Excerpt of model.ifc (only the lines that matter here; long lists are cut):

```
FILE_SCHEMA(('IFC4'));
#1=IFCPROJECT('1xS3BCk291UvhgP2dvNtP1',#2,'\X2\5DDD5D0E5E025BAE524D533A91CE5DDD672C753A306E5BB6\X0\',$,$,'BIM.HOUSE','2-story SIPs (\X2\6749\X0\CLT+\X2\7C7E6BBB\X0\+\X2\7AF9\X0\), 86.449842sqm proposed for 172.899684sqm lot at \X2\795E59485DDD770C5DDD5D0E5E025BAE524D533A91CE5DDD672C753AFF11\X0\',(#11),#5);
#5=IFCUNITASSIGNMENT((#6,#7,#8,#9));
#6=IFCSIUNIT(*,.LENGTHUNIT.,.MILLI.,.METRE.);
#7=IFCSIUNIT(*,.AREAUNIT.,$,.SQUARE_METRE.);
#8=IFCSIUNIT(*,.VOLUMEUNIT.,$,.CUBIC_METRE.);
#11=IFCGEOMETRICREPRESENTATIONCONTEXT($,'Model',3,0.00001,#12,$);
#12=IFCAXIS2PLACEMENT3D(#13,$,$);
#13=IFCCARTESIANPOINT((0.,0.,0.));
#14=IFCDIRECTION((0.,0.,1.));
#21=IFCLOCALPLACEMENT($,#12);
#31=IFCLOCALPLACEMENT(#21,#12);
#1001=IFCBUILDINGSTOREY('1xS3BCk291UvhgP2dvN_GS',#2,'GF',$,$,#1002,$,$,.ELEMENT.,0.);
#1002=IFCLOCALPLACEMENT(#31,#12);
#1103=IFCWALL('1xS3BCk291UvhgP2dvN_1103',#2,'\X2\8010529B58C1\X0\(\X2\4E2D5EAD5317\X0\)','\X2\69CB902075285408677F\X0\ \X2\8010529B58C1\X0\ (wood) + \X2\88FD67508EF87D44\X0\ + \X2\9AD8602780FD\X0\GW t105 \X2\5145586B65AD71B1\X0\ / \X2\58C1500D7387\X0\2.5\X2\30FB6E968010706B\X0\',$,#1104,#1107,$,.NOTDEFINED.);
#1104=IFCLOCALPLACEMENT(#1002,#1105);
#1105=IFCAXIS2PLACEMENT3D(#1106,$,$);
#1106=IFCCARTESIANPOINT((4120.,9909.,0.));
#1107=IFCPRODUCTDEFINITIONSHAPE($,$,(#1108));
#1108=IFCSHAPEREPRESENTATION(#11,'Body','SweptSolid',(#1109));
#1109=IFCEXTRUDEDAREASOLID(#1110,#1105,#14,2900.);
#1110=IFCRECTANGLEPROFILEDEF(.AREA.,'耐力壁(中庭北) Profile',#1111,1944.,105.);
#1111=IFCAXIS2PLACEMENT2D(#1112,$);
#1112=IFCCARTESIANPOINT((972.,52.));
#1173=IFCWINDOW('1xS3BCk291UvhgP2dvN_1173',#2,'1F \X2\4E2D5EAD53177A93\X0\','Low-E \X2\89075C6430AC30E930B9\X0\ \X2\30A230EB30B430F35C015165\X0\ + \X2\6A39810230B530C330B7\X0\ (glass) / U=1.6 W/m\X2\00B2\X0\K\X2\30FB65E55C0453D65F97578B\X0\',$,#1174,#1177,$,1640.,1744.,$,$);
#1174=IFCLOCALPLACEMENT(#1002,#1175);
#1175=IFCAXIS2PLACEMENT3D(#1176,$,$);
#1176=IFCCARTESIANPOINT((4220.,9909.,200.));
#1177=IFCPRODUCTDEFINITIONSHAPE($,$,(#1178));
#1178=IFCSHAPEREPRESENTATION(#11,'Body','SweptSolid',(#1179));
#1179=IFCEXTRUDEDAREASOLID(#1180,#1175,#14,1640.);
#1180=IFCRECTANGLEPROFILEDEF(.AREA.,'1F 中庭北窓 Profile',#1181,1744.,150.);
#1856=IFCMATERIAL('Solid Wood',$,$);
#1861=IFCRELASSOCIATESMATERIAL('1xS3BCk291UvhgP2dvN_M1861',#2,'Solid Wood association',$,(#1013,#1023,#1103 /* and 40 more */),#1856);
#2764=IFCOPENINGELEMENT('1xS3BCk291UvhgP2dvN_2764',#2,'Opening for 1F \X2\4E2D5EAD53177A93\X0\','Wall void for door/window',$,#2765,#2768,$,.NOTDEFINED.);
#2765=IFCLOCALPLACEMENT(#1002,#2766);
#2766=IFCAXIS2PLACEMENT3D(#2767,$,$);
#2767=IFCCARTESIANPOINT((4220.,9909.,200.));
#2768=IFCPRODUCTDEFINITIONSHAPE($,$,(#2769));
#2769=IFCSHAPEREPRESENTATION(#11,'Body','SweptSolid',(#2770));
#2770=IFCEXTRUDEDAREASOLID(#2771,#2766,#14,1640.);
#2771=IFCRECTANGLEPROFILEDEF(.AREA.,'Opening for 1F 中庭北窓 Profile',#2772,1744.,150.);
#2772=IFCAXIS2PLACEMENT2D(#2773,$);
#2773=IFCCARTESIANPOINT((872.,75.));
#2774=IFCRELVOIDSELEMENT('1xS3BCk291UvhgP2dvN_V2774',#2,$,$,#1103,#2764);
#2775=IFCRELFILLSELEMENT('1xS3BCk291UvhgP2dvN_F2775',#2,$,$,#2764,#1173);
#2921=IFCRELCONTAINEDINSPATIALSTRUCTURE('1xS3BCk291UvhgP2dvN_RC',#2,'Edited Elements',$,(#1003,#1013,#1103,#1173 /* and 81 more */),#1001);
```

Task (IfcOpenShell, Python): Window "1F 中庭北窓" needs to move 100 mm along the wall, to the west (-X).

```python
import ifcopenshell
import ifcopenshell.api.geometry
import ifcopenshell.util.placement
import ifcopenshell.util.unit

model = ifcopenshell.open("model.ifc")
unit_scale = ifcopenshell.util.unit.calculate_unit_scale(model)

window = model.by_id(1173)
opening = window.FillsVoids[0].RelatingOpeningElement
wall = opening.VoidsElements[0].RelatingBuildingElement

wall_matrix = ifcopenshell.util.placement.get_local_placement(wall.ObjectPlacement)
shift = wall_matrix[:3, 0] * -0.1 / unit_scale
before = ifcopenshell.util.placement.get_local_placement(window.ObjectPlacement)[:3, 3].copy()

# The window is not placed relative to its opening, so move both.
for product in (opening, window):
    matrix = ifcopenshell.util.placement.get_local_placement(product.ObjectPlacement)
    matrix[:3, 3] += shift
    ifcopenshell.api.geometry.edit_object_placement(model, product=product, matrix=matrix, is_si=False)

after = ifcopenshell.util.placement.get_local_placement(window.ObjectPlacement)[:3, 3]
print("window moved by", (after - before).round(3) + 0.0)

model.write("model_edited.ifc")
```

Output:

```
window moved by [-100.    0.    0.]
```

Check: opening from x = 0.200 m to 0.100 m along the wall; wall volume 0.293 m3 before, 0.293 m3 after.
